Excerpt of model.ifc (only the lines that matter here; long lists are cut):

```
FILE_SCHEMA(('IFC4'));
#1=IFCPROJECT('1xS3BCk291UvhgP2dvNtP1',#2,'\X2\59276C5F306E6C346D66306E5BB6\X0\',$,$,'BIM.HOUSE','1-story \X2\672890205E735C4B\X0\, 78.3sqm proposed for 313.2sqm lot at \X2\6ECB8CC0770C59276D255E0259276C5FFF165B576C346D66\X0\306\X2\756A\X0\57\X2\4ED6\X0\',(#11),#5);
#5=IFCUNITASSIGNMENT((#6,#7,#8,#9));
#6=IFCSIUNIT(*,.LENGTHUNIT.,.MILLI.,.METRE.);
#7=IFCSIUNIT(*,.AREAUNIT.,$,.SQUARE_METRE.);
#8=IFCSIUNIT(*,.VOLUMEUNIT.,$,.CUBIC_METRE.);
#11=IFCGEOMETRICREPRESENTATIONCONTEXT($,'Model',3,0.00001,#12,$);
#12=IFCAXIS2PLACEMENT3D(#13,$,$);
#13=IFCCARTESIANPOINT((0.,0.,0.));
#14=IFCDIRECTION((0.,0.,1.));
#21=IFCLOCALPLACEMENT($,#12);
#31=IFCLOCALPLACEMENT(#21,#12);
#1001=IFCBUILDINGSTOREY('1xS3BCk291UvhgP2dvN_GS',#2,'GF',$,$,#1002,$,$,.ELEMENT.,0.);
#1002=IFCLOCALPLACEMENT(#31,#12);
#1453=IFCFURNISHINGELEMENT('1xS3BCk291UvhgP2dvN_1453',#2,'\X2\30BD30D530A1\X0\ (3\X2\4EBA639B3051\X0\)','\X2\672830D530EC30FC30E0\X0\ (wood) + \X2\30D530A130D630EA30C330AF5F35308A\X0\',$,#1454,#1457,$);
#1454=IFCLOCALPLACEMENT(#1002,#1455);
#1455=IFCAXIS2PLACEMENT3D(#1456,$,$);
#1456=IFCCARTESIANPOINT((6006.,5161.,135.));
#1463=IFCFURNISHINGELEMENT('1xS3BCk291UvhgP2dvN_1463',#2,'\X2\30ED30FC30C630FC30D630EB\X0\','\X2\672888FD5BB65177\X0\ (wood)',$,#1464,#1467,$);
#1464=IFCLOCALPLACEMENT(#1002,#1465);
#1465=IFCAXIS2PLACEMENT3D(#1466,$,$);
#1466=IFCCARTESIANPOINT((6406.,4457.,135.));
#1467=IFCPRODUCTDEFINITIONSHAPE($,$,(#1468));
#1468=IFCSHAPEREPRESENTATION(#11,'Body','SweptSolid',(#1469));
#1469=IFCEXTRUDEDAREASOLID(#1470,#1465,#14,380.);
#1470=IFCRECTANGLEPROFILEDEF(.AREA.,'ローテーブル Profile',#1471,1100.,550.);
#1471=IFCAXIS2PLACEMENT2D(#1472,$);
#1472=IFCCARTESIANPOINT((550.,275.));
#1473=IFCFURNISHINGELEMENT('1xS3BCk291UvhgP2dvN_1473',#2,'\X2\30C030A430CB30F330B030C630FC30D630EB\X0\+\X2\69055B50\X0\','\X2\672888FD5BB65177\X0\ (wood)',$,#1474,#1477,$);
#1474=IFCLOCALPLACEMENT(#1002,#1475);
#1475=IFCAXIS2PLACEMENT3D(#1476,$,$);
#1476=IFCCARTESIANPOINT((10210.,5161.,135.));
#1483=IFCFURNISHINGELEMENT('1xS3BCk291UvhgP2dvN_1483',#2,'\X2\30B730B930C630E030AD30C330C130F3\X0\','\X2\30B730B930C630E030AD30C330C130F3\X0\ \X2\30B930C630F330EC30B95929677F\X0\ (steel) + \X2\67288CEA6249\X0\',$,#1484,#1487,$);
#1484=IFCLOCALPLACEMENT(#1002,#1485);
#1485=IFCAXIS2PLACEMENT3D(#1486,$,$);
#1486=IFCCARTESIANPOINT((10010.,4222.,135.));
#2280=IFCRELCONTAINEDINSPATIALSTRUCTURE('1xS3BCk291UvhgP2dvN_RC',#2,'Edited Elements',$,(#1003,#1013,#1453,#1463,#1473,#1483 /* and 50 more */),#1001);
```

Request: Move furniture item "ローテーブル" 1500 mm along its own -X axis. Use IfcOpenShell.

```python
import ifcopenshell
import ifcopenshell.api.geometry
import ifcopenshell.util.placement

model = ifcopenshell.open("model.ifc")

item = model.by_guid("1xS3BCk291UvhgP2dvN_1463")
matrix = ifcopenshell.util.placement.get_local_placement(item.ObjectPlacement)
matrix[:3, 3] -= matrix[:3, 0] * 1500.0
ifcopenshell.api.geometry.edit_object_placement(model, product=item, matrix=matrix, is_si=False)

print(ifcopenshell.util.placement.get_local_placement(item.ObjectPlacement).round(3) + 0.0)

model.write("model_v2.ifc")
```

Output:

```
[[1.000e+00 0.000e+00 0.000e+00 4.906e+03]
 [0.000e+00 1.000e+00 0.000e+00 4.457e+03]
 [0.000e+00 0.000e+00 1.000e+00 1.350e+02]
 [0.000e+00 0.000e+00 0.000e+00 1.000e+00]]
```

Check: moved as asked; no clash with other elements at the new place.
